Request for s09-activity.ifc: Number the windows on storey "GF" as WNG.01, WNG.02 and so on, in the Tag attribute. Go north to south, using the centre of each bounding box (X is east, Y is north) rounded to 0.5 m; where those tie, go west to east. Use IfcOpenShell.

First a look at what the model holds.

```python
import ifcopenshell
import ifcopenshell.util.element
import ifcopenshell.util.placement

model = ifcopenshell.open("s09-activity.ifc")
print(model.schema)
storey = next(s for s in model.by_type("IfcBuildingStorey") if s.Name == "GF")
windows = [e for e in ifcopenshell.util.element.get_decomposition(storey) if e.is_a("IfcWindow")]
for e in sorted(windows, key=lambda e: e.id()):
    origin = ifcopenshell.util.placement.get_local_placement(e.ObjectPlacement)[:3, 3]
    print(e.id(), e.Tag, e.Name, origin.round(2) + 0.0, sep=" | ")
```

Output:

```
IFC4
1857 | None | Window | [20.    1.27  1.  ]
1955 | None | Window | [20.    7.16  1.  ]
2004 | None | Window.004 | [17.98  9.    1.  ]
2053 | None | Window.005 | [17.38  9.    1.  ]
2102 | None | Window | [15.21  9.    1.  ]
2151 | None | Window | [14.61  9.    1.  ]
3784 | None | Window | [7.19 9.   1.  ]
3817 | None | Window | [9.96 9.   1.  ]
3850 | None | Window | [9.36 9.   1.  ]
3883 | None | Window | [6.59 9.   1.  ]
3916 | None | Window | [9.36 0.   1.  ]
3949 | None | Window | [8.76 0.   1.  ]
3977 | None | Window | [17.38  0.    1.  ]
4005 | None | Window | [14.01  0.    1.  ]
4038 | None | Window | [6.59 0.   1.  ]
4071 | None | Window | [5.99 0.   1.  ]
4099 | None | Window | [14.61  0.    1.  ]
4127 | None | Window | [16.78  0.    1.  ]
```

```python
import ifcopenshell
import ifcopenshell.geom
import ifcopenshell.util.element
import ifcopenshell.util.shape

model = ifcopenshell.open("s09-activity.ifc")
settings = ifcopenshell.geom.settings()
settings.set("use-world-coords", True)


def centre(element):
    shape = ifcopenshell.geom.create_shape(settings, element)
    return ifcopenshell.util.shape.get_bbox_centroid(shape.geometry)


storey = next(s for s in model.by_type("IfcBuildingStorey") if s.Name == "GF")
windows = [e for e in ifcopenshell.util.element.get_decomposition(storey) if e.is_a("IfcWindow")]

# Insertion points can sit at a corner or the storey origin, so sort by the geometry (in metres).
centres = {e: centre(e) for e in windows}
windows.sort(key=lambda e: (-round(centres[e][1] / 0.5), centres[e][0]))

for i, e in enumerate(windows, start=1):
    number = f"WNG.{i:02d}"
    e.Tag = number
    print(e.id(), number)

model.write("s09-activity_rev.ifc")
```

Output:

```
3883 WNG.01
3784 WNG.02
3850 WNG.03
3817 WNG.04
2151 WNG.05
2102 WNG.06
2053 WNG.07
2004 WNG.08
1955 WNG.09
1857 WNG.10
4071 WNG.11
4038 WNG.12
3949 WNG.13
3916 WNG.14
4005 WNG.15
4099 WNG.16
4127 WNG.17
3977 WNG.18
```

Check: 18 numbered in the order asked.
